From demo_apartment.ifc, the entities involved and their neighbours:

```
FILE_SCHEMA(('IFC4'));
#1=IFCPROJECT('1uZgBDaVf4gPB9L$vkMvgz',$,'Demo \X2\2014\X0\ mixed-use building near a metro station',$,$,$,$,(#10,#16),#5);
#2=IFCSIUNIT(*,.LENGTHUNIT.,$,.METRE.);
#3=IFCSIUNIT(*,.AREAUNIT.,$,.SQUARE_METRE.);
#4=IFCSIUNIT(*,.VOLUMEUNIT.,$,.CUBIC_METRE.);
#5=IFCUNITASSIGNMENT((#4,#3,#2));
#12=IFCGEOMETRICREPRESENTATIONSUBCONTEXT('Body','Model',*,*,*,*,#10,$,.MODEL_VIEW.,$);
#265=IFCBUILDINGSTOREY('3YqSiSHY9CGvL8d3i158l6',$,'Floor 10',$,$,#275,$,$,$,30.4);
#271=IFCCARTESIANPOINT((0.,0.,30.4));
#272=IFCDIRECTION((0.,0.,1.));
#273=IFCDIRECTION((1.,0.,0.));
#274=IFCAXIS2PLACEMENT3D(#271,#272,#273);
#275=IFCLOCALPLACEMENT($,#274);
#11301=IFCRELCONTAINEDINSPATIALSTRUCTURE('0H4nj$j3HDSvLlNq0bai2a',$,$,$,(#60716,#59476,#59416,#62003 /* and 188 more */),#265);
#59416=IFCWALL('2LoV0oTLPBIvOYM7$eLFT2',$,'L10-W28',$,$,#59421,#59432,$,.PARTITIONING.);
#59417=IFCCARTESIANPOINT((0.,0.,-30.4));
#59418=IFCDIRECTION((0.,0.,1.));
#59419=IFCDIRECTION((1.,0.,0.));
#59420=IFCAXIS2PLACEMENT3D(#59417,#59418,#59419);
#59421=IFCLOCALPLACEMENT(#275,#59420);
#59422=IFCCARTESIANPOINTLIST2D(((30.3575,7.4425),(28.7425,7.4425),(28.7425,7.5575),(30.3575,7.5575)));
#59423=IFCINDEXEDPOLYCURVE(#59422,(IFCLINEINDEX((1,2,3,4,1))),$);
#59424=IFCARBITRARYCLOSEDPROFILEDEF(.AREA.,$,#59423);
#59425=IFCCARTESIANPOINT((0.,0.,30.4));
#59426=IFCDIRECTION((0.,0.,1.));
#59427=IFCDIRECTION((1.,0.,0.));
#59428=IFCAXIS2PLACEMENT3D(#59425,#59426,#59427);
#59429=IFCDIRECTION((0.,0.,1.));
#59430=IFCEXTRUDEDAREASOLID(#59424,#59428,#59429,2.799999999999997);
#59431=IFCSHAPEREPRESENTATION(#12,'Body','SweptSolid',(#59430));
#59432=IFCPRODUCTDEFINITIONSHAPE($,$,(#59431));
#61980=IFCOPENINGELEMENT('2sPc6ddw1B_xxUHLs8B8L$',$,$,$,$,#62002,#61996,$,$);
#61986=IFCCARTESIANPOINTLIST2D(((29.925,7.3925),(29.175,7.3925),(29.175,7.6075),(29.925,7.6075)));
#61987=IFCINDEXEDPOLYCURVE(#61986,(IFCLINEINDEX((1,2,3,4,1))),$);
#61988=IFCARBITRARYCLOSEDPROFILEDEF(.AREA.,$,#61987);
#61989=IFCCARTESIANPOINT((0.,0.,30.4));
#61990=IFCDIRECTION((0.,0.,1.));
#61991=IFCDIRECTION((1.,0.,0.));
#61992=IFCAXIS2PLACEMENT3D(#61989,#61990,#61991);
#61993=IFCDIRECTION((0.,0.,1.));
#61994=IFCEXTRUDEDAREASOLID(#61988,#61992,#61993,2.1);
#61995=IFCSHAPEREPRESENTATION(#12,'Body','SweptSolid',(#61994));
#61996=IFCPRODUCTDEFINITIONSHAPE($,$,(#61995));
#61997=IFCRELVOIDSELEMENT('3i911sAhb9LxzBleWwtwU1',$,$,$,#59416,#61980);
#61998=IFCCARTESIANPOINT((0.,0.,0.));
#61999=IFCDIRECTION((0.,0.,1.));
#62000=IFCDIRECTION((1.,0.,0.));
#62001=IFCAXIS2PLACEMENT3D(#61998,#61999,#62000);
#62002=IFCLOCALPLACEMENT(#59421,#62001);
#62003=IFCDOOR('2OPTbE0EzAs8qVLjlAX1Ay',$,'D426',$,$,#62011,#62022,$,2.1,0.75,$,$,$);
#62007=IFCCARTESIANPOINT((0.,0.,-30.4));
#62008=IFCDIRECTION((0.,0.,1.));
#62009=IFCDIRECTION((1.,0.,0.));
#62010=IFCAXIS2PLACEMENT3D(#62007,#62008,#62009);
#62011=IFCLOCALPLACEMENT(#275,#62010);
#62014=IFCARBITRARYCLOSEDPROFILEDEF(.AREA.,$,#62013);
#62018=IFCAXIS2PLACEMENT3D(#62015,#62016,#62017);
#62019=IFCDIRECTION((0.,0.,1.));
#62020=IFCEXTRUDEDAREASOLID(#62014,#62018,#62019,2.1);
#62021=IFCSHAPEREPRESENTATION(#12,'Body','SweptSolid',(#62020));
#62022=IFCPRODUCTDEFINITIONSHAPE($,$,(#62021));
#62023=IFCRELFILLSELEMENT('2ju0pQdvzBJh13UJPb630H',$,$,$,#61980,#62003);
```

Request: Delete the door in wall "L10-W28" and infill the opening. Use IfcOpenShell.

```python
import ifcopenshell
import ifcopenshell.api.feature
import ifcopenshell.api.root
import ifcopenshell.geom
import ifcopenshell.util.shape

model = ifcopenshell.open("demo_apartment.ifc")
settings = ifcopenshell.geom.settings()


def volume(element):
    """Net volume in cubic metres, openings subtracted."""
    shape = ifcopenshell.geom.create_shape(settings, element)
    return ifcopenshell.util.shape.get_volume(shape.geometry)


door = model.by_guid("2OPTbE0EzAs8qVLjlAX1Ay")
opening = door.FillsVoids[0].RelatingOpeningElement
wall = opening.VoidsElements[0].RelatingBuildingElement
before = volume(wall)

ifcopenshell.api.root.remove_product(model, product=door)
ifcopenshell.api.feature.remove_feature(model, feature=opening)

after = volume(wall)

print(f"wall volume {before:.3f} -> {after:.3f} m3")

model.write("demo_apartment_v2.ifc")
```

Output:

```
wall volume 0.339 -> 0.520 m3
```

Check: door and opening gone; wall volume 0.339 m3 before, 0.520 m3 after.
